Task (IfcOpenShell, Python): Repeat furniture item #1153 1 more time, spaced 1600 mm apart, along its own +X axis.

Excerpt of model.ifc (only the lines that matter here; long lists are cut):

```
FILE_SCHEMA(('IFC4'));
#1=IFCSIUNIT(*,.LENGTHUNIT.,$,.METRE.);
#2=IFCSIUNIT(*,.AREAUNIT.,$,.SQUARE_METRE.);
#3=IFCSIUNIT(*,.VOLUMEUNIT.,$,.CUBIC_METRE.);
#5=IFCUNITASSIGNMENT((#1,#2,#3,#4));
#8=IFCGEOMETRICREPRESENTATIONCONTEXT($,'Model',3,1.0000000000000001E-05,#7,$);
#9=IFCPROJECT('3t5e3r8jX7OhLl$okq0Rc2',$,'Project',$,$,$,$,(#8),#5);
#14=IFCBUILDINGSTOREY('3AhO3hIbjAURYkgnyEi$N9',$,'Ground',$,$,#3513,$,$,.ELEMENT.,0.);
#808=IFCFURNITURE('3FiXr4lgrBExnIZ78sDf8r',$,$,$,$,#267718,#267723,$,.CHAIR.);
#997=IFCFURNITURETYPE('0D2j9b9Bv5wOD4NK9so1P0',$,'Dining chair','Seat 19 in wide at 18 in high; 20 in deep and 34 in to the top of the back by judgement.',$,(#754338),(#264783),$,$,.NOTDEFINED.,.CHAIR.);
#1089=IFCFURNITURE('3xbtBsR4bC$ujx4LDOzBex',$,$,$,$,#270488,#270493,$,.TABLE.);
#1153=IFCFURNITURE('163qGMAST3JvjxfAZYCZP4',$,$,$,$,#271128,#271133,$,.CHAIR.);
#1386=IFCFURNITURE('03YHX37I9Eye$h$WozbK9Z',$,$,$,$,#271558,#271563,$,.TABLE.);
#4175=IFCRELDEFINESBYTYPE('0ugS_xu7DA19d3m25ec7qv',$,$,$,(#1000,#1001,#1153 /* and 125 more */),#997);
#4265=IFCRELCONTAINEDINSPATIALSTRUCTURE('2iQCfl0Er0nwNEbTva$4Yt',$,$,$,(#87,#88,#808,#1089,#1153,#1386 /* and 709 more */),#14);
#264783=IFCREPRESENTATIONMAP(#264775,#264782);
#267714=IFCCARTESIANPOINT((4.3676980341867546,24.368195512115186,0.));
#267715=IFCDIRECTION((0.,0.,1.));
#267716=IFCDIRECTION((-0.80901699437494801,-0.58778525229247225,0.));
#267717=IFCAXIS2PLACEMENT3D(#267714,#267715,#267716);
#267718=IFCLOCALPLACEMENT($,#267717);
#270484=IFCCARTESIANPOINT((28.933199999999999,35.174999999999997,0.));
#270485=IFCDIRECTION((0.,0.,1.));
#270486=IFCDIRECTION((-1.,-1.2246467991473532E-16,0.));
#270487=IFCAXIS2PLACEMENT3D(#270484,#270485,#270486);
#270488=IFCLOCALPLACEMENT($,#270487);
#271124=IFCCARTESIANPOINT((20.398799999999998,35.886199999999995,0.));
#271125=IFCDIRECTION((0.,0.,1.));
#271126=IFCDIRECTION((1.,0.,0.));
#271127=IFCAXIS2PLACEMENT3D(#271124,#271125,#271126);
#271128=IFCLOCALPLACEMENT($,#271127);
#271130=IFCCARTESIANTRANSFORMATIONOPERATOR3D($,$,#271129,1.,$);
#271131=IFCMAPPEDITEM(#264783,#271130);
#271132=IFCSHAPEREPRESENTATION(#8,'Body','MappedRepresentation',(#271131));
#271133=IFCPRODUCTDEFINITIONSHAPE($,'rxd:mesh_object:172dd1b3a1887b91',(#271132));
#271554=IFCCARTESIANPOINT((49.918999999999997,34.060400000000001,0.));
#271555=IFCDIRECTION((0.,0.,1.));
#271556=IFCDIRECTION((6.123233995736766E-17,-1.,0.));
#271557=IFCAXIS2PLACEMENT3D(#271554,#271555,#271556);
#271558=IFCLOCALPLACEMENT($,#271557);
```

```python
import ifcopenshell
import ifcopenshell.api.geometry
import ifcopenshell.api.root
import ifcopenshell.util.element
import ifcopenshell.util.placement
import ifcopenshell.util.unit

model = ifcopenshell.open("model.ifc")
unit_scale = ifcopenshell.util.unit.calculate_unit_scale(model)

source = model.by_id(1153)
base = ifcopenshell.util.placement.get_local_placement(source.ObjectPlacement)
step = base[:3, 0] * 1.6 / unit_scale

for i in range(1, 2):
    copy = ifcopenshell.api.root.copy_class(model, product=source)
    copy.Representation = ifcopenshell.util.element.copy_deep(
        model, source.Representation, exclude=["IfcGeometricRepresentationContext", "IfcRepresentationMap"]
    )
    matrix = base.copy()
    matrix[:3, 3] += i * step
    print("added at", matrix[:3, 3].round(3) + 0.0)
    ifcopenshell.api.geometry.edit_object_placement(model, product=copy, matrix=matrix, is_si=False)

model.write("model_rev.ifc")
```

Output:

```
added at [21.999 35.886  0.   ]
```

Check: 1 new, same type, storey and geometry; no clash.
